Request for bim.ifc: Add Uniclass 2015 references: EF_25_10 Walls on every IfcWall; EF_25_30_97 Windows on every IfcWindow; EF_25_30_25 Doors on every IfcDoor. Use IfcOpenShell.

First a look at what the model holds.

```python
import ifcopenshell

model = ifcopenshell.open("bim.ifc")
print(model.schema)
print("classifications:", [c.Name for c in model.by_type("IfcClassification")])
for ifc_class in ("IfcDoor", "IfcRoof", "IfcStair", "IfcWall", "IfcWindow"):
    print(ifc_class, len(model.by_type(ifc_class)))
```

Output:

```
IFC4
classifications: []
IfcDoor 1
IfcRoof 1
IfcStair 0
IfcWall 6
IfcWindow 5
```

```python
import ifcopenshell
import ifcopenshell.api.classification

model = ifcopenshell.open("bim.ifc")

system = ifcopenshell.api.classification.add_classification(model, classification="Uniclass 2015")

codes = {
    "IfcWall": ("EF_25_10", "Walls"),
    "IfcWindow": ("EF_25_30_97", "Windows"),
    "IfcDoor": ("EF_25_30_25", "Doors"),
}
for ifc_class, (code, name) in codes.items():
    products = model.by_type(ifc_class)
    ifcopenshell.api.classification.add_reference(
        model, products=products, classification=system, identification=code, name=name
    )
    print(code, len(products))

model.write("bim_v2.ifc")
```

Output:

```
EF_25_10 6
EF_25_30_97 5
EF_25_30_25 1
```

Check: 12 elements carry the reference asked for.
